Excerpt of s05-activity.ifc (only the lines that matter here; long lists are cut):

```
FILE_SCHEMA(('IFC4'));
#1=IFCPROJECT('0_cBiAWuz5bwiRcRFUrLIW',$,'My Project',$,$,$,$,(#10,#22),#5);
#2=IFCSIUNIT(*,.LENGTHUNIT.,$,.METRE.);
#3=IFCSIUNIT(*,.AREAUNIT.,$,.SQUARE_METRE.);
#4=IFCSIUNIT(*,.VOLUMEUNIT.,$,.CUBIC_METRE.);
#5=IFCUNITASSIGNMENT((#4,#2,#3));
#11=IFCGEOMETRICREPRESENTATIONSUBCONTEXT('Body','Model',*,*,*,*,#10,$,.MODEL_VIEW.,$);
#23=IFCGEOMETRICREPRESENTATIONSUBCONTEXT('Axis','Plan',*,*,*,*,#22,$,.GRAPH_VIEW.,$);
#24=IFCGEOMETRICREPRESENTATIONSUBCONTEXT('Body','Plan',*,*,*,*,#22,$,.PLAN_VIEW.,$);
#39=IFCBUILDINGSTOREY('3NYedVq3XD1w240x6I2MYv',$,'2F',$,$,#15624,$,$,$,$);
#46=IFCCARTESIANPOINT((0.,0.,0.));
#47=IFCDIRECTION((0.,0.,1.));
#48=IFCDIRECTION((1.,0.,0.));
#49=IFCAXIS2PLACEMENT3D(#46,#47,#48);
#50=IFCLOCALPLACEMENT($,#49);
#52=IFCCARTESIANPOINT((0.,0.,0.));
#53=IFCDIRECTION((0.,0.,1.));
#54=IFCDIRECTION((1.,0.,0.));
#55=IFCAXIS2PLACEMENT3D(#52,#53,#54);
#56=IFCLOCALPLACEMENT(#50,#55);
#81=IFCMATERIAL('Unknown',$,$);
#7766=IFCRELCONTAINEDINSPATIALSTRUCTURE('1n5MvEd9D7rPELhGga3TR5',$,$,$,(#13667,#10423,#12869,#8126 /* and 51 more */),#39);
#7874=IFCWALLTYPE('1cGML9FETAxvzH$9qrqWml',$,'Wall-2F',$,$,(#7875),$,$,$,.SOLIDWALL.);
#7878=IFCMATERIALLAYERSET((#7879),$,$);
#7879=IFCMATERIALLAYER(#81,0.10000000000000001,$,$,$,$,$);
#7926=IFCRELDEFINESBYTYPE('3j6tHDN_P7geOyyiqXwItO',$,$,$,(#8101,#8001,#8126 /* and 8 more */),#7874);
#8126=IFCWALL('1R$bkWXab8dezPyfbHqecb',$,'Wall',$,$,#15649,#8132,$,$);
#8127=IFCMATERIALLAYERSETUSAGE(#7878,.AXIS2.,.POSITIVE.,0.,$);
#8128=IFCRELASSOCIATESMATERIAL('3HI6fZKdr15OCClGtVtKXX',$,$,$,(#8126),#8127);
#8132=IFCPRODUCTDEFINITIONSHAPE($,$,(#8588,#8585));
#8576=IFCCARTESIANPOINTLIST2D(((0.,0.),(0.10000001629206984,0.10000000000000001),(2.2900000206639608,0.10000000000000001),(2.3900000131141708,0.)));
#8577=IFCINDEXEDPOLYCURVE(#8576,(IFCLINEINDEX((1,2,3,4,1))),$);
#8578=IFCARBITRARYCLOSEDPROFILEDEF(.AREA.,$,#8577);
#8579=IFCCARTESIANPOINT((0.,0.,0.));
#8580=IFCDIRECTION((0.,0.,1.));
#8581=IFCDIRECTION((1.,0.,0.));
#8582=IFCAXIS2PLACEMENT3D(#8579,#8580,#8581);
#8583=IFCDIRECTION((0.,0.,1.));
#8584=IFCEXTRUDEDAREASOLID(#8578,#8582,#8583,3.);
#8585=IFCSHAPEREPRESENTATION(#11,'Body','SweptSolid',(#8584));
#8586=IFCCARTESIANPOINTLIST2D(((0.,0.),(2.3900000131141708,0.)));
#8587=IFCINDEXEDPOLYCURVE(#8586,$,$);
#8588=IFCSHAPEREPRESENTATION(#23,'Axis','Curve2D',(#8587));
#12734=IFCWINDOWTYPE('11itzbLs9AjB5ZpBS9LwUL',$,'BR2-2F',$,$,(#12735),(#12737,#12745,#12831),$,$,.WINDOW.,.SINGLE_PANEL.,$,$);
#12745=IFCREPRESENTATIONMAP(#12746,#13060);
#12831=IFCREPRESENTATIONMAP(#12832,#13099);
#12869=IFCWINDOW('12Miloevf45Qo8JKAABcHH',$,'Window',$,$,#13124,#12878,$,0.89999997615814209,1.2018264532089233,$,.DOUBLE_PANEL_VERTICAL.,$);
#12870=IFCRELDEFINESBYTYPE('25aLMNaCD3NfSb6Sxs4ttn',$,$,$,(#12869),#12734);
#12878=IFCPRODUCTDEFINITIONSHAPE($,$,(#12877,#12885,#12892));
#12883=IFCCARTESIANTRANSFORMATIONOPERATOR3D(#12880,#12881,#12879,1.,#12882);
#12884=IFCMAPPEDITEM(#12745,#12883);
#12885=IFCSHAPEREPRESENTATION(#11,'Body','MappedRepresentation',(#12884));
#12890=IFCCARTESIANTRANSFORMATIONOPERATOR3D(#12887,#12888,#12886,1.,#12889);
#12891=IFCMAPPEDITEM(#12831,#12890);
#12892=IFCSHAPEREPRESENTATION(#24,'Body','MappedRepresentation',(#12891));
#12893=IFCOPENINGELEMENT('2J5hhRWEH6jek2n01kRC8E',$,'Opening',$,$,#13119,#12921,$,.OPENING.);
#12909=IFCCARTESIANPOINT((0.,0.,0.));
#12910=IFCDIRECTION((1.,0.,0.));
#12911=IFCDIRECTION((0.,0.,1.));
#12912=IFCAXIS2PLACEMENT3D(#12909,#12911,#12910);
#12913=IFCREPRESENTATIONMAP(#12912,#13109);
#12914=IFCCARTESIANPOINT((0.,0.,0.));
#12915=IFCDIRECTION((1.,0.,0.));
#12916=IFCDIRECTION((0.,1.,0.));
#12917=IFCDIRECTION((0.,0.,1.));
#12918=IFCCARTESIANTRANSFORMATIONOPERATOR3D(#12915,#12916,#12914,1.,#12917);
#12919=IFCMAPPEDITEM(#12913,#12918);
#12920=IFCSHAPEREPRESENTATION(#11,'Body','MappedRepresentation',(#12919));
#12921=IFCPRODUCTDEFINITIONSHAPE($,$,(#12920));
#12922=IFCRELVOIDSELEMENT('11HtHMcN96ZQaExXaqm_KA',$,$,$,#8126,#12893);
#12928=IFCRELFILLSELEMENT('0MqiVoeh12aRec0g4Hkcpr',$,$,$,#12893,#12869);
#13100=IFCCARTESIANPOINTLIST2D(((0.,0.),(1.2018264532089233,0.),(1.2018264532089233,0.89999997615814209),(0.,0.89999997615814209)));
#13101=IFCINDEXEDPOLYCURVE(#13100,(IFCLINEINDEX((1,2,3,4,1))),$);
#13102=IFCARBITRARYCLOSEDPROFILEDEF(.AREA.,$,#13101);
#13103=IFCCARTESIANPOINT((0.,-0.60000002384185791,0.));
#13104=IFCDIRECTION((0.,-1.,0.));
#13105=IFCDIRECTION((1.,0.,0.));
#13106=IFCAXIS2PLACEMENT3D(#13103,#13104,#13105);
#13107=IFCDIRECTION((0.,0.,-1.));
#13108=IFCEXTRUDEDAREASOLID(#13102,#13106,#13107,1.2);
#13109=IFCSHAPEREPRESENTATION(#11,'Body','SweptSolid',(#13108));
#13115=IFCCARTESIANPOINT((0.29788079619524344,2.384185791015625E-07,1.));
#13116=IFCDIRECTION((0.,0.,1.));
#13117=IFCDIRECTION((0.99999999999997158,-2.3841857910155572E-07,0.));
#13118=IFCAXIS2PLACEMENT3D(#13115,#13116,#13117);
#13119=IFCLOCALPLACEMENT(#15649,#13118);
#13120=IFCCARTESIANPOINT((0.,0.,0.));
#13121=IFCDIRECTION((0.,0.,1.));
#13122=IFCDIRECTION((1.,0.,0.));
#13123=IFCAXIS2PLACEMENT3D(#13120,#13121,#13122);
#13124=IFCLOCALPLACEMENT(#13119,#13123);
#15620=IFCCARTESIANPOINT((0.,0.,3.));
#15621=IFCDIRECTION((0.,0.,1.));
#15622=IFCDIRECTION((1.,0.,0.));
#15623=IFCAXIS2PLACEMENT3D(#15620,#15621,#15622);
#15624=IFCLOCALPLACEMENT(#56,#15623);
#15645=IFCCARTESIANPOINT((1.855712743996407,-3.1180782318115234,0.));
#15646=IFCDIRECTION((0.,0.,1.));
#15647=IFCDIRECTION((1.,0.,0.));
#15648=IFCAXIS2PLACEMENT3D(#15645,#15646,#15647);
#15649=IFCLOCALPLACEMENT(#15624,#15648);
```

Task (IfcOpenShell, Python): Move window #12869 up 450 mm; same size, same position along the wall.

```python
import numpy as np
import ifcopenshell
import ifcopenshell.api.geometry
import ifcopenshell.util.placement
import ifcopenshell.util.unit

model = ifcopenshell.open("s05-activity.ifc")
unit_scale = ifcopenshell.util.unit.calculate_unit_scale(model)

window = model.by_guid("12Miloevf45Qo8JKAABcHH")
opening = window.FillsVoids[0].RelatingOpeningElement
dz = 0.45 / unit_scale

shift = np.array([0.0, 0.0, dz])
# The window is placed relative to its opening, so it follows when the opening moves.
matrix = ifcopenshell.util.placement.get_local_placement(opening.ObjectPlacement)
matrix[:3, 3] += shift
ifcopenshell.api.geometry.edit_object_placement(
    model, product=opening, matrix=matrix, is_si=False, should_transform_children=True
)

print(f"moved by {dz * unit_scale:+.3f} m")

model.write("s05-activity_v2.ifc")
```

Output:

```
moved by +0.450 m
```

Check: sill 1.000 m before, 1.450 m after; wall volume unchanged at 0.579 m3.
